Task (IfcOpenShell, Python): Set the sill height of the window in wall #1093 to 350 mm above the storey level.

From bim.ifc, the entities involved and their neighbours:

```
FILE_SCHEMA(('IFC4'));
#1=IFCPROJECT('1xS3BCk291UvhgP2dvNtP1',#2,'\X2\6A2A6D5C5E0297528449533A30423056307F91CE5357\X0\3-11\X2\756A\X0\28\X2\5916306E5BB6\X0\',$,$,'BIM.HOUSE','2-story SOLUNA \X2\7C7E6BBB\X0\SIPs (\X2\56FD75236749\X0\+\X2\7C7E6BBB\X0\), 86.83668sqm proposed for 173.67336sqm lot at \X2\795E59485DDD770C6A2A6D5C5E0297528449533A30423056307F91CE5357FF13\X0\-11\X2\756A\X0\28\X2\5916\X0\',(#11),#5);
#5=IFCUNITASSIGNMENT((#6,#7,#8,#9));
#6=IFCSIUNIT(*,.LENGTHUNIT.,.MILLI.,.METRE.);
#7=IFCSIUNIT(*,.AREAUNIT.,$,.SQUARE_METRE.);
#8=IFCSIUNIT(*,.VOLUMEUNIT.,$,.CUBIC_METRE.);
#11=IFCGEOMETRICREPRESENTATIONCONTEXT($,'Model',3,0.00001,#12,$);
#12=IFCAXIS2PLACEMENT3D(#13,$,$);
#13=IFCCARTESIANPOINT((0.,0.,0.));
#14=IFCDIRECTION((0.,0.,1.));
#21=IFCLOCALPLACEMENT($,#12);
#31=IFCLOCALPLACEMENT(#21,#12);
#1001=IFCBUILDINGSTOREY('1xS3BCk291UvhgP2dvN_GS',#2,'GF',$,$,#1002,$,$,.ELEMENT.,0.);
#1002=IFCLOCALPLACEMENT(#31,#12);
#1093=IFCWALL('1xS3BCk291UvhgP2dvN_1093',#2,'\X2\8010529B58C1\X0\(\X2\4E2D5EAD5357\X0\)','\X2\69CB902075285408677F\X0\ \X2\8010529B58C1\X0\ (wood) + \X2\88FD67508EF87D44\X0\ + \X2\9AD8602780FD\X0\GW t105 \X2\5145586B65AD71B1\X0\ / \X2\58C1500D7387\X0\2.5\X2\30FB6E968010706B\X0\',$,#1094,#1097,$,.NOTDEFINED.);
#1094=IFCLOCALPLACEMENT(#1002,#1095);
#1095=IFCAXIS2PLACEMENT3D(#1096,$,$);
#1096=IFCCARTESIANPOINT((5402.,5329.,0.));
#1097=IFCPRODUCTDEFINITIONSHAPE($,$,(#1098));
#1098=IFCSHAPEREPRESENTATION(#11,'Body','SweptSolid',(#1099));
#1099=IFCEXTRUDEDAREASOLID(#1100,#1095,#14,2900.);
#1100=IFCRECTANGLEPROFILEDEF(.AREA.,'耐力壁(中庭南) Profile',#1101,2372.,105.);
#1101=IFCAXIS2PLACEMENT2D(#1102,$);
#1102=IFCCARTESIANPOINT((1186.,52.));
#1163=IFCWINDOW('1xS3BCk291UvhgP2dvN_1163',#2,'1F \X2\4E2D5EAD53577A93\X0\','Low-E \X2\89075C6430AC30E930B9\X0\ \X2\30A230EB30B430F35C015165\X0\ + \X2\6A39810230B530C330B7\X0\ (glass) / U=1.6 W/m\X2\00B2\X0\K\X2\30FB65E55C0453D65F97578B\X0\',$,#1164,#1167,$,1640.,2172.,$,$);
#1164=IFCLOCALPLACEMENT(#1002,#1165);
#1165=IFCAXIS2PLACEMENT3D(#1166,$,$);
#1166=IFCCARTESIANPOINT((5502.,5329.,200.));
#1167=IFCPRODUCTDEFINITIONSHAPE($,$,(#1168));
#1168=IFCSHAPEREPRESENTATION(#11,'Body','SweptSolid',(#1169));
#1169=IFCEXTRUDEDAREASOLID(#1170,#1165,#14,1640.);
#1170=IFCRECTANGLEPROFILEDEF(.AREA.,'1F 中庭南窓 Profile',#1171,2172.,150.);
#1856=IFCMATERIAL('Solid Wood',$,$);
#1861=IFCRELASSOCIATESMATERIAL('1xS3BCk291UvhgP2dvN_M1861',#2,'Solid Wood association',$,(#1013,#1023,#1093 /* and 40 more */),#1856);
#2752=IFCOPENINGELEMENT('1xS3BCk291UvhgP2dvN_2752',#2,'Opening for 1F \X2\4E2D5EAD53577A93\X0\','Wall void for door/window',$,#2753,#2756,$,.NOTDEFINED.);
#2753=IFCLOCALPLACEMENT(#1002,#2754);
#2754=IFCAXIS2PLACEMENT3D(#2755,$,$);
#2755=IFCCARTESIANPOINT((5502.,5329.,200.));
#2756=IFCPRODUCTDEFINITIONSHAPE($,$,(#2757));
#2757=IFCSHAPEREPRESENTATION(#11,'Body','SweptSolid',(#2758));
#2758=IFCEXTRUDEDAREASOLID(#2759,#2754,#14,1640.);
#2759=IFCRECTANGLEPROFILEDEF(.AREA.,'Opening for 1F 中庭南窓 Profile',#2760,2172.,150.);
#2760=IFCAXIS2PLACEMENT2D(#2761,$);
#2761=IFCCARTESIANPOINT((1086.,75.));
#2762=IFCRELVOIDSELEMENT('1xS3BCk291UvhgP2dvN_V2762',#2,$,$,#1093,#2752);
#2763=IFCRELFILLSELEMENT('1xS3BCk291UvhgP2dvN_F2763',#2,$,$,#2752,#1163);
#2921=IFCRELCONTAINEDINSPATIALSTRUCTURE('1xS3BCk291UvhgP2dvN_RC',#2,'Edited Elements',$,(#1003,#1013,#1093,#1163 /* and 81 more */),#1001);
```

```python
import numpy as np
import ifcopenshell
import ifcopenshell.api.geometry
import ifcopenshell.geom
import ifcopenshell.util.element
import ifcopenshell.util.placement
import ifcopenshell.util.shape
import ifcopenshell.util.unit

model = ifcopenshell.open("bim.ifc")
unit_scale = ifcopenshell.util.unit.calculate_unit_scale(model)

window = model.by_guid("1xS3BCk291UvhgP2dvN_1163")
opening = window.FillsVoids[0].RelatingOpeningElement
storey = ifcopenshell.util.element.get_container(window, ifc_class="IfcBuildingStorey")
level = ifcopenshell.util.placement.get_local_placement(storey.ObjectPlacement)[2, 3]

# The opening's origin need not be at the sill, so measure its lowest point.
shape = ifcopenshell.geom.create_shape(ifcopenshell.geom.settings(), opening)
bottom = ifcopenshell.util.shape.get_shape_bottom_elevation(shape, shape.geometry) / unit_scale
dz = level + 0.35 / unit_scale - bottom

shift = np.array([0.0, 0.0, dz])
# The window is not placed relative to its opening, so move both.
for product in (opening, window):
    matrix = ifcopenshell.util.placement.get_local_placement(product.ObjectPlacement)
    matrix[:3, 3] += shift
    ifcopenshell.api.geometry.edit_object_placement(model, product=product, matrix=matrix, is_si=False)

print(f"moved by {dz * unit_scale:+.3f} m")

model.write("bim_edited.ifc")
```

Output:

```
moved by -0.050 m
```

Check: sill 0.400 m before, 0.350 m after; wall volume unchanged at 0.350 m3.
